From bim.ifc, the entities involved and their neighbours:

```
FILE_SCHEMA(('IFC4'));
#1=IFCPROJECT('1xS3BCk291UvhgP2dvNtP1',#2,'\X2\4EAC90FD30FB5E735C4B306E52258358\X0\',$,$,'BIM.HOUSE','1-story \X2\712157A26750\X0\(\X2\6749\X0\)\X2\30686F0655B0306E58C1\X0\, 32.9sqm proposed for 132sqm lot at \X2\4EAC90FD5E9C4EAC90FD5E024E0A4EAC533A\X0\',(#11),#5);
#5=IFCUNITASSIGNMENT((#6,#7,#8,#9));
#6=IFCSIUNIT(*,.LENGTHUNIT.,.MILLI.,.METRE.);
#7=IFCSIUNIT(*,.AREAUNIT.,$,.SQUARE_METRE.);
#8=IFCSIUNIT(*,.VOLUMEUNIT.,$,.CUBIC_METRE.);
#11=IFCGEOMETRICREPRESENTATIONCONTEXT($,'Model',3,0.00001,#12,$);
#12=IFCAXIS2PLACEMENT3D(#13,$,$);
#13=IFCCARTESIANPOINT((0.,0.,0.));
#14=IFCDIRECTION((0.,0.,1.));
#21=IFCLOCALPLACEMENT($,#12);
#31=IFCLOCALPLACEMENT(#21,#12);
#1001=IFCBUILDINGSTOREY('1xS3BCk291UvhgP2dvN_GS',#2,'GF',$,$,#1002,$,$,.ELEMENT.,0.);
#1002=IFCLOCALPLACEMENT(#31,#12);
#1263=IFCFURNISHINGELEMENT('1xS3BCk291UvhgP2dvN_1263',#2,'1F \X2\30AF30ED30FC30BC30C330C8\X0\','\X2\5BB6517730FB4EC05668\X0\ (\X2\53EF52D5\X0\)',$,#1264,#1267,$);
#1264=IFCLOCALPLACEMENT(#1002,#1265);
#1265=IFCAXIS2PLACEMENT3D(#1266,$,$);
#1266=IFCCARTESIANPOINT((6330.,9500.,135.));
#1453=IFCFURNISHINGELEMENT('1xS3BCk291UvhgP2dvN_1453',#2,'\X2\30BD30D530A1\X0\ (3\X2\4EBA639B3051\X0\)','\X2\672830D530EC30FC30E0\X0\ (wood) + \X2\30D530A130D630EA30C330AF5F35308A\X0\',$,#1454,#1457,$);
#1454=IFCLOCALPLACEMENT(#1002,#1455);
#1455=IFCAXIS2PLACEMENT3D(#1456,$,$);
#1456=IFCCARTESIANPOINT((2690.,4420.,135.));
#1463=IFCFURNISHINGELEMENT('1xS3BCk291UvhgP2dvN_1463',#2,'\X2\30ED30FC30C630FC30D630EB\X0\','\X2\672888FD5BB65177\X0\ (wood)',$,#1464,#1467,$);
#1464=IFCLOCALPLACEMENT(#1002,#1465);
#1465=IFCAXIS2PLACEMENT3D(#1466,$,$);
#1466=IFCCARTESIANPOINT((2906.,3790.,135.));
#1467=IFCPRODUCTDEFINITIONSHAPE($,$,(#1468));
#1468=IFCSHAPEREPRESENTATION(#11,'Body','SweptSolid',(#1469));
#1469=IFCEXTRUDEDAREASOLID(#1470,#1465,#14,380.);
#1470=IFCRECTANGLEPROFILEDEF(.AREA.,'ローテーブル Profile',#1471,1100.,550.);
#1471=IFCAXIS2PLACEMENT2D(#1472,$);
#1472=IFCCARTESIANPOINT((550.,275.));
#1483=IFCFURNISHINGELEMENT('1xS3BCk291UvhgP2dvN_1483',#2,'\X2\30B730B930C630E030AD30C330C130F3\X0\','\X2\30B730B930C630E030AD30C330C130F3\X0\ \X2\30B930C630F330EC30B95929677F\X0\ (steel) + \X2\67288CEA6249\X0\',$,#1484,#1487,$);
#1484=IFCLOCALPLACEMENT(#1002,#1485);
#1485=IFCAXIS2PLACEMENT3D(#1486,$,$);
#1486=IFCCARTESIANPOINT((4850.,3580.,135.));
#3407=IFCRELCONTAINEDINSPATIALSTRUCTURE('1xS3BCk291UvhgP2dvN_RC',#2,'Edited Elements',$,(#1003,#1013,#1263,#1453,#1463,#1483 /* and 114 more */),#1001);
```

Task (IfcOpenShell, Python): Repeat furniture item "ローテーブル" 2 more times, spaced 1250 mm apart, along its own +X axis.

```python
import ifcopenshell
import ifcopenshell.api.geometry
import ifcopenshell.api.root
import ifcopenshell.util.element
import ifcopenshell.util.placement

model = ifcopenshell.open("bim.ifc")


def reuse_history(source, copy):
    """copy_class also copies each property set's owner history, people and application; keep the originals."""
    for rel in copy.IsDefinedBy:
        if rel.is_a("IfcRelDefinesByProperties") and (history := rel.RelatingPropertyDefinition.OwnerHistory):
            rel.RelatingPropertyDefinition.OwnerHistory = source.OwnerHistory
            ifcopenshell.util.element.remove_deep2(model, history)


source = model.by_guid("1xS3BCk291UvhgP2dvN_1463")
base = ifcopenshell.util.placement.get_local_placement(source.ObjectPlacement)
step = base[:3, 0] * 1250.0

for i in range(1, 3):
    copy = ifcopenshell.api.root.copy_class(model, product=source)
    copy.Representation = ifcopenshell.util.element.copy_deep(
        model, source.Representation, exclude=["IfcGeometricRepresentationContext", "IfcRepresentationMap"]
    )
    reuse_history(source, copy)
    matrix = base.copy()
    matrix[:3, 3] += i * step
    print("added at", matrix[:3, 3].round(3) + 0.0)
    ifcopenshell.api.geometry.edit_object_placement(model, product=copy, matrix=matrix, is_si=False)

model.write("bim_edited.ifc")
```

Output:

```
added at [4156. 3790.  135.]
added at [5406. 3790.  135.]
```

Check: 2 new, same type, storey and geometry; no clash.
